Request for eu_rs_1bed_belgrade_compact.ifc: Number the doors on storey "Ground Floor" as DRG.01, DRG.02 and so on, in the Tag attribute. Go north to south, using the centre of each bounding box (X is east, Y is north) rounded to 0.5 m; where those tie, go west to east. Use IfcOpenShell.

First a look at what the model holds.

```python
import ifcopenshell
import ifcopenshell.util.element
import ifcopenshell.util.placement

model = ifcopenshell.open("eu_rs_1bed_belgrade_compact.ifc")
print(model.schema)
storey = next(s for s in model.by_type("IfcBuildingStorey") if s.Name == "Ground Floor")
doors = [e for e in ifcopenshell.util.element.get_decomposition(storey) if e.is_a("IfcDoor")]
for e in sorted(doors, key=lambda e: e.id()):
    origin = ifcopenshell.util.placement.get_local_placement(e.ObjectPlacement)[:3, 3]
    print(e.id(), e.Tag, e.Name, origin.round(2) + 0.0, sep=" | ")
```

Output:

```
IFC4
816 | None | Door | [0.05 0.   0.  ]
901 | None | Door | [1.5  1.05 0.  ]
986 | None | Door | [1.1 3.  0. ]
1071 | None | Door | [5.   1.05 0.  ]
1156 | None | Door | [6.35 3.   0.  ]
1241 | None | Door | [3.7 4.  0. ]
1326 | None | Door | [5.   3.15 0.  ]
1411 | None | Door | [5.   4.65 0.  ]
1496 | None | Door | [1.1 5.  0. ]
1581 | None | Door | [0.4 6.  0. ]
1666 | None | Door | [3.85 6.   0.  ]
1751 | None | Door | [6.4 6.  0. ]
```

```python
import ifcopenshell
import ifcopenshell.geom
import ifcopenshell.util.element
import ifcopenshell.util.shape

model = ifcopenshell.open("eu_rs_1bed_belgrade_compact.ifc")
settings = ifcopenshell.geom.settings()
settings.set("use-world-coords", True)


def centre(element):
    shape = ifcopenshell.geom.create_shape(settings, element)
    return ifcopenshell.util.shape.get_bbox_centroid(shape.geometry)


storey = next(s for s in model.by_type("IfcBuildingStorey") if s.Name == "Ground Floor")
doors = [e for e in ifcopenshell.util.element.get_decomposition(storey) if e.is_a("IfcDoor")]

# Insertion points can sit at a corner or the storey origin, so sort by the geometry (in metres).
centres = {e: centre(e) for e in doors}
doors.sort(key=lambda e: (-round(centres[e][1] / 0.5), centres[e][0]))

for i, e in enumerate(doors, start=1):
    number = f"DRG.{i:02d}"
    e.Tag = number
    print(e.id(), number)

model.write("eu_rs_1bed_belgrade_compact_edited.ifc")
```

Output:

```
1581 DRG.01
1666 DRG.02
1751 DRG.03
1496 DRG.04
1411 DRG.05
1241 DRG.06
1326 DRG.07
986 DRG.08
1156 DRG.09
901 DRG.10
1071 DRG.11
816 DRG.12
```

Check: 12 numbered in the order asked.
